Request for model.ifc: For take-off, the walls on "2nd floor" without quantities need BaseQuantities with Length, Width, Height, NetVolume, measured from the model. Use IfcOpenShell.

First a look at what the model holds.

```python
import ifcopenshell
import ifcopenshell.util.element
import ifcopenshell.util.unit

model = ifcopenshell.open("model.ifc")
print(model.schema)
for unit_type in ("LENGTHUNIT", "AREAUNIT", "VOLUMEUNIT"):
    print(unit_type, ifcopenshell.util.unit.calculate_unit_scale(model, unit_type))
storey = next(s for s in model.by_type("IfcBuildingStorey") if s.Name == "2nd floor")
walls = [e for e in ifcopenshell.util.element.get_decomposition(storey) if e.is_a("IfcWall")]
for e in sorted(walls, key=lambda e: e.id()):
    print(e.id(), e.is_a(), e.Name, list(ifcopenshell.util.element.get_psets(e, qtos_only=True)), sep=" | ")
```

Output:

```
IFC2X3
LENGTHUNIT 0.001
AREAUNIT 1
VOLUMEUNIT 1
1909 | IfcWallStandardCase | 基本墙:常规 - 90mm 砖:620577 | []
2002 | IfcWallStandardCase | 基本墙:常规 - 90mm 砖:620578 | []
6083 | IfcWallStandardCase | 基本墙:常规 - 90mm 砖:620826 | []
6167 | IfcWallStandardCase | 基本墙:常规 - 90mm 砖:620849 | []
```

```python
import ifcopenshell
import ifcopenshell.api.pset
import ifcopenshell.geom
import ifcopenshell.util.element
import ifcopenshell.util.shape
import ifcopenshell.util.unit

model = ifcopenshell.open("model.ifc")
unit_scale = ifcopenshell.util.unit.calculate_unit_scale(model)
volume_scale = ifcopenshell.util.unit.calculate_unit_scale(model, "VOLUMEUNIT")
settings = ifcopenshell.geom.settings()

storey = next(s for s in model.by_type("IfcBuildingStorey") if s.Name == "2nd floor")
walls = [e for e in ifcopenshell.util.element.get_decomposition(storey) if e.is_a("IfcWall")]

for e in sorted(walls, key=lambda e: e.id()):
    if ifcopenshell.util.element.get_psets(e, qtos_only=True, should_inherit=False):
        continue
    # Geometry comes back in metres, in the element's own axes.
    shape = ifcopenshell.geom.create_shape(settings, e)
    values = {
        "Length": ifcopenshell.util.shape.get_x(shape.geometry) / unit_scale,
        "Width": ifcopenshell.util.shape.get_y(shape.geometry) / unit_scale,
        "Height": ifcopenshell.util.shape.get_z(shape.geometry) / unit_scale,
        "NetVolume": ifcopenshell.util.shape.get_volume(shape.geometry) / volume_scale,
    }
    qto = ifcopenshell.api.pset.add_qto(model, product=e, name="BaseQuantities")
    ifcopenshell.api.pset.edit_qto(model, qto=qto, properties=values)
    print(e.id(), {k: round(v, 3) for k, v in values.items()})

model.write("model-out.ifc")
```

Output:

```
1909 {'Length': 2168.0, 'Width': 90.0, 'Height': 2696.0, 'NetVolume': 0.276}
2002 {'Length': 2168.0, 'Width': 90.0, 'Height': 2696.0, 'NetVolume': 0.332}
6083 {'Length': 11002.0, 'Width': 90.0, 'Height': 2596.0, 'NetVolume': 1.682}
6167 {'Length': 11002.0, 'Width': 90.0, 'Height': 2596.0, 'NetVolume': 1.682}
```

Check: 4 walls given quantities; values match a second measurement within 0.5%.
